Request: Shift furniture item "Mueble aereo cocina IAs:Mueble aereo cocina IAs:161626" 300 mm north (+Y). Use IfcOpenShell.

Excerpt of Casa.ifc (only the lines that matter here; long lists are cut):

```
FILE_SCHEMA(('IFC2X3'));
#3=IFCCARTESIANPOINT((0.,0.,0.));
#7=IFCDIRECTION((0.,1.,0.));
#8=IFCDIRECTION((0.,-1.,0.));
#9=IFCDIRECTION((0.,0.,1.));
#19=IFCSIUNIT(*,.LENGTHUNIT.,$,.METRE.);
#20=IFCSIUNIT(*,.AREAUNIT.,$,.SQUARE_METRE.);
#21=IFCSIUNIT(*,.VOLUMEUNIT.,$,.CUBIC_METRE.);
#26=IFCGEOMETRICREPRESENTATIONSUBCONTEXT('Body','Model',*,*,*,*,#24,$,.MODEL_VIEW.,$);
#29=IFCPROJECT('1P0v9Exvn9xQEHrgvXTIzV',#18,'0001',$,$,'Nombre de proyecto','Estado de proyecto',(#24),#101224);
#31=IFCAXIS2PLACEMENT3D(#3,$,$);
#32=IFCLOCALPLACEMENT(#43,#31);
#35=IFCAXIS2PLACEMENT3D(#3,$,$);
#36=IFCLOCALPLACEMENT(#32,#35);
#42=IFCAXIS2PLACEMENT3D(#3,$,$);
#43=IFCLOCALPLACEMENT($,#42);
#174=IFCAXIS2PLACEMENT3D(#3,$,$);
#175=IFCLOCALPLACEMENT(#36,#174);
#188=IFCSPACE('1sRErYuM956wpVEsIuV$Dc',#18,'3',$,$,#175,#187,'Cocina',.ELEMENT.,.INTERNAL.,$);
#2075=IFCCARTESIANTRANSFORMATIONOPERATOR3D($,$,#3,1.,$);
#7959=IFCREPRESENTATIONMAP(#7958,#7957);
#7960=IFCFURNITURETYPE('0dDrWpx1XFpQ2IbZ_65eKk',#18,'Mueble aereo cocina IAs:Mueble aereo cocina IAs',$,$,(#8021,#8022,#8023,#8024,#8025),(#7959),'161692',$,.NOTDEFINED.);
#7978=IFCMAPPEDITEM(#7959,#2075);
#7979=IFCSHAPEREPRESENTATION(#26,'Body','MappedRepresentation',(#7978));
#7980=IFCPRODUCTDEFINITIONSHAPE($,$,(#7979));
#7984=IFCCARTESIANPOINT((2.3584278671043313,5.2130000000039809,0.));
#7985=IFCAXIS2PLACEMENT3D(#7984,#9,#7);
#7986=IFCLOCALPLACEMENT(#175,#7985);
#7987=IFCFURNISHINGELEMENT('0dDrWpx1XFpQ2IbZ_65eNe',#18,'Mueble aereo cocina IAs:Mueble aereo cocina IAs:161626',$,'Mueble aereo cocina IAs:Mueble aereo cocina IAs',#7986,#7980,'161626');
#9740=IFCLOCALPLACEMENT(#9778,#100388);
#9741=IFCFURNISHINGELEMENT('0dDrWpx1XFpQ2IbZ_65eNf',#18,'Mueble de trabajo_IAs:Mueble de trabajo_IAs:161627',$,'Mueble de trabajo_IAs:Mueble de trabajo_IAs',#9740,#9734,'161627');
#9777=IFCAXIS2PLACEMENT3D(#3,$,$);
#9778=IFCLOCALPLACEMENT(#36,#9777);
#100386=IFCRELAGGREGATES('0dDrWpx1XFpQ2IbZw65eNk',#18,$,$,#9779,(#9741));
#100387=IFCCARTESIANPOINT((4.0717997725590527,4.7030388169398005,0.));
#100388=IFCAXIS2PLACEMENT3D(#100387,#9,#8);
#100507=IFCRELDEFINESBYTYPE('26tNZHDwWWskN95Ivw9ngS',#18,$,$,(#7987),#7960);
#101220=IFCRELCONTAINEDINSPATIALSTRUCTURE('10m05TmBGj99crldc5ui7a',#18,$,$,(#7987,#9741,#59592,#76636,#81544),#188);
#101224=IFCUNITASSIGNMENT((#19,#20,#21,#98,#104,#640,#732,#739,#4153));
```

```python
import ifcopenshell
import ifcopenshell.api.geometry
import ifcopenshell.util.placement
import ifcopenshell.util.unit

model = ifcopenshell.open("Casa.ifc")
unit_scale = ifcopenshell.util.unit.calculate_unit_scale(model)

item = model.by_id(7987)
matrix = ifcopenshell.util.placement.get_local_placement(item.ObjectPlacement)
matrix[1, 3] += 0.3 / unit_scale
ifcopenshell.api.geometry.edit_object_placement(model, product=item, matrix=matrix, is_si=False)

print(ifcopenshell.util.placement.get_local_placement(item.ObjectPlacement).round(3) + 0.0)

model.write("Casa_v2.ifc")
```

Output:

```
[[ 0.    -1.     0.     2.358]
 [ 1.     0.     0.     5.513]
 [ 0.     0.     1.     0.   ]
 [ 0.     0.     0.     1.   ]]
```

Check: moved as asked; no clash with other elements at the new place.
